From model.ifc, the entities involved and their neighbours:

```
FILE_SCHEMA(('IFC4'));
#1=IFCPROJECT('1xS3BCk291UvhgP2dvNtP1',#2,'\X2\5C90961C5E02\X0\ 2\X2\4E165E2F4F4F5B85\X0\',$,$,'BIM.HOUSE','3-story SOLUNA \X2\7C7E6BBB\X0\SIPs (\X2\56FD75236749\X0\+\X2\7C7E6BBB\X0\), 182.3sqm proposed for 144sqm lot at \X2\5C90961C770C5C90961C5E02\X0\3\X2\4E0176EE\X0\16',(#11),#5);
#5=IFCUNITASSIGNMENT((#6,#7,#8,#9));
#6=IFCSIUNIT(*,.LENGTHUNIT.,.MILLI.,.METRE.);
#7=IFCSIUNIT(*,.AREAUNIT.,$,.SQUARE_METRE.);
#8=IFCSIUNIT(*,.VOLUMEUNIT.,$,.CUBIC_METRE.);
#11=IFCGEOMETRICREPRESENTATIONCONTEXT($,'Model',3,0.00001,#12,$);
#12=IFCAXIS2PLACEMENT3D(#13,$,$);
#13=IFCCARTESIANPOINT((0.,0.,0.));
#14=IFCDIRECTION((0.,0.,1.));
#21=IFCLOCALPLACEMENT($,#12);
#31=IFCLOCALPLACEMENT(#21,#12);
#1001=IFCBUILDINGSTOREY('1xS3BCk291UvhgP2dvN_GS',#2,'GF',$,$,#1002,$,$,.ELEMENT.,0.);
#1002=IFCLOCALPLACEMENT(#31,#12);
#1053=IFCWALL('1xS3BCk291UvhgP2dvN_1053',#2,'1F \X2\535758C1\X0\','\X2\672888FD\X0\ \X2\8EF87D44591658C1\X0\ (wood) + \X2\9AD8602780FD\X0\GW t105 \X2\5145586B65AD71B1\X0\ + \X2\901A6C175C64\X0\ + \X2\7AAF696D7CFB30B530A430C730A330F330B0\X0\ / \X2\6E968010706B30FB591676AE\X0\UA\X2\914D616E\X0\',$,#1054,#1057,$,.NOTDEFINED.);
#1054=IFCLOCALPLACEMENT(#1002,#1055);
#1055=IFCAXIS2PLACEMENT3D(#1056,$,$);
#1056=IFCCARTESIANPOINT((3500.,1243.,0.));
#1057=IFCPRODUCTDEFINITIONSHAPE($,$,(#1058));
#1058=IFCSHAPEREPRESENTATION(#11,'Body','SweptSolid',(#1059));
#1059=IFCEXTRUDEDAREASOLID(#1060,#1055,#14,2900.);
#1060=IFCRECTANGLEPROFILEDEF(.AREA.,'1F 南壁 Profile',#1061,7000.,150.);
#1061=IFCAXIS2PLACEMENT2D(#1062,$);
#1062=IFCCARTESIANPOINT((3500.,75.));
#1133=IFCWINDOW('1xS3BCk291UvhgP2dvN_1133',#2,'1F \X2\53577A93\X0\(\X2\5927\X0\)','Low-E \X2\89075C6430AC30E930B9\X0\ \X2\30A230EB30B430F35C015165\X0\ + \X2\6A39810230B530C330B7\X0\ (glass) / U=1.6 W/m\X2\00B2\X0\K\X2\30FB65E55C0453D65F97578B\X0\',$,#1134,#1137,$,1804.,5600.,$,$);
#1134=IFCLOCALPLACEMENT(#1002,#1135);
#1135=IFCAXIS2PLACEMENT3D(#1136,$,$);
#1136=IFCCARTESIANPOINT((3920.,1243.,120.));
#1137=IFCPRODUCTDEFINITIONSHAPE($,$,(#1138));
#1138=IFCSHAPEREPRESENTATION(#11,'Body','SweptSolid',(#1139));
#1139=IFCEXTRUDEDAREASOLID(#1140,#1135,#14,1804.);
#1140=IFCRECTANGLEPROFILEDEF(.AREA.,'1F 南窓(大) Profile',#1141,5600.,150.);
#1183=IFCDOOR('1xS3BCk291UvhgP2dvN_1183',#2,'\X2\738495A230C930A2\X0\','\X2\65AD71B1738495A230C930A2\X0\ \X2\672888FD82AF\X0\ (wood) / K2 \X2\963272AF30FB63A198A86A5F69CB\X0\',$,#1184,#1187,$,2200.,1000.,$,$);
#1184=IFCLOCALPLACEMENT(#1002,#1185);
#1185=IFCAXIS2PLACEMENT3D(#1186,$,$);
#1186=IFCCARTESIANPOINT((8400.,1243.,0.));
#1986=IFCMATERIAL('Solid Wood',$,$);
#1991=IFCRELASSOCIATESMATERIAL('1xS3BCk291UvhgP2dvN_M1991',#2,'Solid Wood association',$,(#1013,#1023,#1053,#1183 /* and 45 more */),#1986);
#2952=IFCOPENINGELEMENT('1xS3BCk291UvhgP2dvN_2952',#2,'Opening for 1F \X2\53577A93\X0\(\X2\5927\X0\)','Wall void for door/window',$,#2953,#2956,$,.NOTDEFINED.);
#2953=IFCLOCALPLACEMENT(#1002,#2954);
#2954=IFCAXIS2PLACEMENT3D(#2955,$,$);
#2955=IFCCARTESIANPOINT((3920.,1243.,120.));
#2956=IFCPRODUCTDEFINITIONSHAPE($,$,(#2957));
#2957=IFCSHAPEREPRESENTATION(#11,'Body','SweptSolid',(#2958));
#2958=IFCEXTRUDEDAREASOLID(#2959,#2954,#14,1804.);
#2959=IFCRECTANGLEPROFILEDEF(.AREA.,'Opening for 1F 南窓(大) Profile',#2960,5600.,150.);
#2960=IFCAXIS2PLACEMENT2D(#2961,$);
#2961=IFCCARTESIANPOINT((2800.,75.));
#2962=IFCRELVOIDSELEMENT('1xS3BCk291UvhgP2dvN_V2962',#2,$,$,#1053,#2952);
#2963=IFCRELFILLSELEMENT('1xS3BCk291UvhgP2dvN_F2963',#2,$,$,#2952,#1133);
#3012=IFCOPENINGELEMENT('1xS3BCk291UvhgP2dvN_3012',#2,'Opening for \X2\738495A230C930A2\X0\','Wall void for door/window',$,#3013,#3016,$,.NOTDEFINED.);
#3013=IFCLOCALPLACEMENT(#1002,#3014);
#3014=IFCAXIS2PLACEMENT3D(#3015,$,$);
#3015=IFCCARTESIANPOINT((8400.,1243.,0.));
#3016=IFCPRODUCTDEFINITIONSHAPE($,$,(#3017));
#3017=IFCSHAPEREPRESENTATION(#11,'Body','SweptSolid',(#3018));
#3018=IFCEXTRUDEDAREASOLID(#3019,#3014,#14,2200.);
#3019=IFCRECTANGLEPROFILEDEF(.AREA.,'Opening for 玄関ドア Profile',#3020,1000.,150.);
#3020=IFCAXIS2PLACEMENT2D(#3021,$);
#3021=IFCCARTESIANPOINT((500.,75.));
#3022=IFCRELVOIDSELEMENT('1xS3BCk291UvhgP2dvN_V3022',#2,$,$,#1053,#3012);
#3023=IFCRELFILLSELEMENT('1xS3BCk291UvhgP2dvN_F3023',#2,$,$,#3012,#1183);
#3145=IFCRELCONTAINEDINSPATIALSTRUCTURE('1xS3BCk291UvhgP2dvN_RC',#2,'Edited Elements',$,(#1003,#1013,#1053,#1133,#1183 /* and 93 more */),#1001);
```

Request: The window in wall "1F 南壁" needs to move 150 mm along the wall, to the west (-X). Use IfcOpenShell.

```python
import ifcopenshell
import ifcopenshell.api.geometry
import ifcopenshell.util.placement
import ifcopenshell.util.unit

model = ifcopenshell.open("model.ifc")
unit_scale = ifcopenshell.util.unit.calculate_unit_scale(model)

window = model.by_id(1133)
opening = window.FillsVoids[0].RelatingOpeningElement
wall = opening.VoidsElements[0].RelatingBuildingElement

wall_matrix = ifcopenshell.util.placement.get_local_placement(wall.ObjectPlacement)
shift = wall_matrix[:3, 0] * -0.15 / unit_scale
before = ifcopenshell.util.placement.get_local_placement(window.ObjectPlacement)[:3, 3].copy()

# The window is not placed relative to its opening, so move both.
for product in (opening, window):
    matrix = ifcopenshell.util.placement.get_local_placement(product.ObjectPlacement)
    matrix[:3, 3] += shift
    ifcopenshell.api.geometry.edit_object_placement(model, product=product, matrix=matrix, is_si=False)

after = ifcopenshell.util.placement.get_local_placement(window.ObjectPlacement)[:3, 3]
print("window moved by", (after - before).round(3) + 0.0)

model.write("model_v2.ifc")
```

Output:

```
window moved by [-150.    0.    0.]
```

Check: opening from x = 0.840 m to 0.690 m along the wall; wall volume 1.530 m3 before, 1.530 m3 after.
